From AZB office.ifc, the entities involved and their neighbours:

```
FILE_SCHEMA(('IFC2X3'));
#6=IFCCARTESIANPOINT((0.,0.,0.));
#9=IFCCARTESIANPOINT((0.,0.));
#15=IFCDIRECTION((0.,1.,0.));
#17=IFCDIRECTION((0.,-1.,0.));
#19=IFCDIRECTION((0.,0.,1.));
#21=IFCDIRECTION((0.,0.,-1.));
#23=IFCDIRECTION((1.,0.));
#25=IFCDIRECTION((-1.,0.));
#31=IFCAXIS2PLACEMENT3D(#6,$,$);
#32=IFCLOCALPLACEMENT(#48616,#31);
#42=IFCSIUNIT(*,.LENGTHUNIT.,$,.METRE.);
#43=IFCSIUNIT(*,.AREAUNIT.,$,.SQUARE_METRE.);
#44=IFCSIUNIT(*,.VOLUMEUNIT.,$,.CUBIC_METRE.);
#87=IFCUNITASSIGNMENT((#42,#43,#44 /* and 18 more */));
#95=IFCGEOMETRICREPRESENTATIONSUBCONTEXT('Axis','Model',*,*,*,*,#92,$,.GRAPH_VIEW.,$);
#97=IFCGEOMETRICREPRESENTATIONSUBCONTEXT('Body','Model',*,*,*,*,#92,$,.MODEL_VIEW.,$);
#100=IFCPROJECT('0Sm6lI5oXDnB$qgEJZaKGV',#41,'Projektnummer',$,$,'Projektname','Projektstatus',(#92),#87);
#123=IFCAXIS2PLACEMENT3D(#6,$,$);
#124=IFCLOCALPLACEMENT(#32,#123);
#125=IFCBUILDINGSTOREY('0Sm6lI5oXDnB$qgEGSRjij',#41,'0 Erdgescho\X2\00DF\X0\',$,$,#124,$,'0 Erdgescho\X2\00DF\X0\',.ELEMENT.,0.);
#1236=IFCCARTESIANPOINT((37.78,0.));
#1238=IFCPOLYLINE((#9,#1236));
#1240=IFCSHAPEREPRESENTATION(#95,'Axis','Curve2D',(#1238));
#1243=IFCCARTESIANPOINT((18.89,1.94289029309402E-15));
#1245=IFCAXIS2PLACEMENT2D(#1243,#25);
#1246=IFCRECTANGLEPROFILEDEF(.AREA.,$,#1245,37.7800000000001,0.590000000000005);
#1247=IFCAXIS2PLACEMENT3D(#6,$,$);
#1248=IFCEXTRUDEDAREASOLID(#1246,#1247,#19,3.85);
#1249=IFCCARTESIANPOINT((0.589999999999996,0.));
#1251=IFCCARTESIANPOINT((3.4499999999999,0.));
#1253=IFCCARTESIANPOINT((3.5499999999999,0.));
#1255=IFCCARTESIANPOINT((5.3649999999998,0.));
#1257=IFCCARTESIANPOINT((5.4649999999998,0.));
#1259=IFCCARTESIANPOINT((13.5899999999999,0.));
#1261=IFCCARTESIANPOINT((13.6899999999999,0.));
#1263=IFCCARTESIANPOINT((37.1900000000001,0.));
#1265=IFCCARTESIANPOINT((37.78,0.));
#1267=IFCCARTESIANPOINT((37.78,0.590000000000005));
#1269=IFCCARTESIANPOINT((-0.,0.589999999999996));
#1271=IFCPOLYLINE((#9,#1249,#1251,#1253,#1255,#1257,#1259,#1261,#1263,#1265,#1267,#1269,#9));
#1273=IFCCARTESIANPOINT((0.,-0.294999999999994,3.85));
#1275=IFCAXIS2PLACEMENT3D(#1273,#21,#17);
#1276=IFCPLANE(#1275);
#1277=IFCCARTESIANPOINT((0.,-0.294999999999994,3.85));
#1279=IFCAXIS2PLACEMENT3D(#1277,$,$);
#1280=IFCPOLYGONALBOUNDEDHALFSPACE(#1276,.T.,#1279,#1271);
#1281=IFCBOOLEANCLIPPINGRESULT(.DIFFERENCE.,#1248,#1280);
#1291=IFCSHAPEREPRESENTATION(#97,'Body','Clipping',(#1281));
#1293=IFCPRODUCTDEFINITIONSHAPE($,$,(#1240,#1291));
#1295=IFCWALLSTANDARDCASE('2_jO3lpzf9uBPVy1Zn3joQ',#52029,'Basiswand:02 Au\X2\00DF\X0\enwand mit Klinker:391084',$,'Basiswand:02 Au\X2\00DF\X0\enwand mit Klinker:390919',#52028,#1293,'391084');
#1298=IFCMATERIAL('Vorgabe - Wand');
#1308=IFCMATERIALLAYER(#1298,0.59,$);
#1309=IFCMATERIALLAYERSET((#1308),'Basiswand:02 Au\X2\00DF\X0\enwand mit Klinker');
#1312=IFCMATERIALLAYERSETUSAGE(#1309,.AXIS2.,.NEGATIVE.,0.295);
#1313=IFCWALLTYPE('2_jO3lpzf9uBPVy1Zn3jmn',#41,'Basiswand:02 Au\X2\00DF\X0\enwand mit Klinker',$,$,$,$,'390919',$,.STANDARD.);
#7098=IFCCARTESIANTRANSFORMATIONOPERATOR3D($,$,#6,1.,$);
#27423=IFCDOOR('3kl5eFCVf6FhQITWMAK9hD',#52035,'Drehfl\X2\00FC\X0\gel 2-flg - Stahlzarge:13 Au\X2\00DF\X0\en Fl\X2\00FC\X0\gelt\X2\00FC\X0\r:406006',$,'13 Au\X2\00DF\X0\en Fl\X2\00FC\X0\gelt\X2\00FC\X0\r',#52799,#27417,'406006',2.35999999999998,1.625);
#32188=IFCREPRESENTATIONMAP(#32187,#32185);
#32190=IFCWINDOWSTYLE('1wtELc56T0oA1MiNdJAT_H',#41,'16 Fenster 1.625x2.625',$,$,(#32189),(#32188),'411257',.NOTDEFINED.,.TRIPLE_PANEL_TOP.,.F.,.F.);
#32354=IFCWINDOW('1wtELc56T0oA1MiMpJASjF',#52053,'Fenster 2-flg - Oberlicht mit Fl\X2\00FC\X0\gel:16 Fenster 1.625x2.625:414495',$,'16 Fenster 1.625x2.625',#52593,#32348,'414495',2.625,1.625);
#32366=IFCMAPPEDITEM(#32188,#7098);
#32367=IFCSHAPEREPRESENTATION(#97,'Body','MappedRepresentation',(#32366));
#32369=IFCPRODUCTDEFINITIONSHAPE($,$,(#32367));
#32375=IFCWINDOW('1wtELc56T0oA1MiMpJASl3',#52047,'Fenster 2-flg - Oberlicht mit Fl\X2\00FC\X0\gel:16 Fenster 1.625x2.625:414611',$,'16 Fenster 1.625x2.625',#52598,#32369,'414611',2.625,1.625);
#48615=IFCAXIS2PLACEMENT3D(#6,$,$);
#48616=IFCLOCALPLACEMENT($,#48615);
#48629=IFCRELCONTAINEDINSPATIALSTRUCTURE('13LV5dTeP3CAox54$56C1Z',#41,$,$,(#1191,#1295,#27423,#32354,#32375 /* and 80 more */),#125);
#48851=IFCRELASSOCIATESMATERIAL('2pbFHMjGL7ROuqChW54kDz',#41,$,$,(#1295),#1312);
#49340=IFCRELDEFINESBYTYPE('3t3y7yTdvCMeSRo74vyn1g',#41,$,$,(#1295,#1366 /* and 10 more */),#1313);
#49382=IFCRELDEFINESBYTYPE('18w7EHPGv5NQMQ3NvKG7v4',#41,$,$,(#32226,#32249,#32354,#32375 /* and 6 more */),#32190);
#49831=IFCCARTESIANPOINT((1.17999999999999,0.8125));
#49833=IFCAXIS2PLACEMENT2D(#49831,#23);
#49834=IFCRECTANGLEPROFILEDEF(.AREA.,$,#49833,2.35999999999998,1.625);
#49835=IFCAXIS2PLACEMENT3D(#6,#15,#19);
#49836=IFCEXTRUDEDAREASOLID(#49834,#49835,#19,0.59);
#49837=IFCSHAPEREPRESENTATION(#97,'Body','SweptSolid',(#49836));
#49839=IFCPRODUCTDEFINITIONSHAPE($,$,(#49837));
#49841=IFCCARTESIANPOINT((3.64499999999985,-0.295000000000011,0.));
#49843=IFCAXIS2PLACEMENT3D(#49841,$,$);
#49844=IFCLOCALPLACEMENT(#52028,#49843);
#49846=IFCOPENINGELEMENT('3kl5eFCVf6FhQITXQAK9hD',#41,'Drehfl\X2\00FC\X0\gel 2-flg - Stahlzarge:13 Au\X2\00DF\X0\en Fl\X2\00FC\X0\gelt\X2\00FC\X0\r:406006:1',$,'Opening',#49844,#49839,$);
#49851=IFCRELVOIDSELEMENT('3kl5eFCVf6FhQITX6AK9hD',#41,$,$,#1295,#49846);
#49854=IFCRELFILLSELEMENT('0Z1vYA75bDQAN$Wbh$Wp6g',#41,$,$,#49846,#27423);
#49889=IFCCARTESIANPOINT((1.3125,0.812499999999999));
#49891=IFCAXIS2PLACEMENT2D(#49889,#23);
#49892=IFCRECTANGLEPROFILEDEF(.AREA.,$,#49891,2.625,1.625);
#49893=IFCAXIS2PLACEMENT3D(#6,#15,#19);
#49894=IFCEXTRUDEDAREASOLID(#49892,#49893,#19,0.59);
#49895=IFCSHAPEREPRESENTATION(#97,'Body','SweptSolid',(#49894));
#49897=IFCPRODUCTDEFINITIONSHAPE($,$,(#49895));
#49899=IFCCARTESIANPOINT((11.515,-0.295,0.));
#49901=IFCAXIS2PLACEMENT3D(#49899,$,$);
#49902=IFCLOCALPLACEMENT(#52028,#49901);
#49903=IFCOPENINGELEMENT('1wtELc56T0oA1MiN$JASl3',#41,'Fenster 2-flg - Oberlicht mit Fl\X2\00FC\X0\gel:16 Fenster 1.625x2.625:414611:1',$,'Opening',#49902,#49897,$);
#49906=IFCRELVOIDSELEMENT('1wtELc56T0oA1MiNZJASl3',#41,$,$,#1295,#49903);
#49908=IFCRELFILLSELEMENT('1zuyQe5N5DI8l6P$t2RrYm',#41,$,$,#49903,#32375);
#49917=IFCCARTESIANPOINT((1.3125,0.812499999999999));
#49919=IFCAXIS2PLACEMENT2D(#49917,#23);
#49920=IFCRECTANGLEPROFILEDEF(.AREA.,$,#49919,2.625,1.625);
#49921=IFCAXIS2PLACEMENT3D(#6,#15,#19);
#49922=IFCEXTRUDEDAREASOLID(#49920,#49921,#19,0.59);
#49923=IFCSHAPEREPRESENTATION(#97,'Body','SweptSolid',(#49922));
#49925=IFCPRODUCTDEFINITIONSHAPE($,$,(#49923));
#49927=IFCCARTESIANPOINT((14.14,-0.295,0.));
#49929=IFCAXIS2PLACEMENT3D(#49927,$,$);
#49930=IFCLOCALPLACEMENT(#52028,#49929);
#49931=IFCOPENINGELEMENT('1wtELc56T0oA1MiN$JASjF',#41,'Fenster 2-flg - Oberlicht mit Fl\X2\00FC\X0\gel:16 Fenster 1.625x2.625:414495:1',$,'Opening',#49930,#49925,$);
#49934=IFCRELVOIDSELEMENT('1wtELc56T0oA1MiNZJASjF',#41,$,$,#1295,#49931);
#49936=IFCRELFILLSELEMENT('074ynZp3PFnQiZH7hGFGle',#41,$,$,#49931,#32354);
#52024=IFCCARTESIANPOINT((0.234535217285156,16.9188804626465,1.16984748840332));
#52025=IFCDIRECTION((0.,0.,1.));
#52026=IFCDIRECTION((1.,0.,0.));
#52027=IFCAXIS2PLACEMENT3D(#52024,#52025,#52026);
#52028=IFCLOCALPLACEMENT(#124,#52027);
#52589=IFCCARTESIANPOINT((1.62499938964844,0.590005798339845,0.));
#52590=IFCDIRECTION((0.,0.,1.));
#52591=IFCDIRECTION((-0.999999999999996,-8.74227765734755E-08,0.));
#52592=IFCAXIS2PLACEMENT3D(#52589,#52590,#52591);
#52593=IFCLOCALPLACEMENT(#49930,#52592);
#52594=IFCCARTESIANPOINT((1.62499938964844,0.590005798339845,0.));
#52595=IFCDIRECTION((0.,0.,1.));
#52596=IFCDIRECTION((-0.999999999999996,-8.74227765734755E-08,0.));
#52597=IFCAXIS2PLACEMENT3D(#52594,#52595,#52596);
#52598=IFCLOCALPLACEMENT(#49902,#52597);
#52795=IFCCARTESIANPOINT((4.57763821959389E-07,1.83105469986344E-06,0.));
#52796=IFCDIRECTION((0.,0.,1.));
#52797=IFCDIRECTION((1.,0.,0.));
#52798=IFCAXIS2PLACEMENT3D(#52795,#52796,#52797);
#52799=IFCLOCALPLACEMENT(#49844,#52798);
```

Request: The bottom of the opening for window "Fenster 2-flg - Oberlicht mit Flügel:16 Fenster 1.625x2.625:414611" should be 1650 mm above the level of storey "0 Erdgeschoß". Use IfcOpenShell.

```python
import numpy as np
import ifcopenshell
import ifcopenshell.api.geometry
import ifcopenshell.geom
import ifcopenshell.util.element
import ifcopenshell.util.placement
import ifcopenshell.util.shape
import ifcopenshell.util.unit

model = ifcopenshell.open("AZB office.ifc")
unit_scale = ifcopenshell.util.unit.calculate_unit_scale(model)

window = model.by_guid("1wtELc56T0oA1MiMpJASl3")
opening = window.FillsVoids[0].RelatingOpeningElement
storey = ifcopenshell.util.element.get_container(window, ifc_class="IfcBuildingStorey")
level = ifcopenshell.util.placement.get_local_placement(storey.ObjectPlacement)[2, 3]

# The opening's origin need not be at the sill, so measure its lowest point.
shape = ifcopenshell.geom.create_shape(ifcopenshell.geom.settings(), opening)
bottom = ifcopenshell.util.shape.get_shape_bottom_elevation(shape, shape.geometry) / unit_scale
dz = level + 1.65 / unit_scale - bottom

shift = np.array([0.0, 0.0, dz])
# The window is placed relative to its opening, so it follows when the opening moves.
matrix = ifcopenshell.util.placement.get_local_placement(opening.ObjectPlacement)
matrix[:3, 3] += shift
ifcopenshell.api.geometry.edit_object_placement(
    model, product=opening, matrix=matrix, is_si=False, should_transform_children=True
)

print(f"moved by {dz * unit_scale:+.3f} m")

model.write("AZB office_rev.ifc")
```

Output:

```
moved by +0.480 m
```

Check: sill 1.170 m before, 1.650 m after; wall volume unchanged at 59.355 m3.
